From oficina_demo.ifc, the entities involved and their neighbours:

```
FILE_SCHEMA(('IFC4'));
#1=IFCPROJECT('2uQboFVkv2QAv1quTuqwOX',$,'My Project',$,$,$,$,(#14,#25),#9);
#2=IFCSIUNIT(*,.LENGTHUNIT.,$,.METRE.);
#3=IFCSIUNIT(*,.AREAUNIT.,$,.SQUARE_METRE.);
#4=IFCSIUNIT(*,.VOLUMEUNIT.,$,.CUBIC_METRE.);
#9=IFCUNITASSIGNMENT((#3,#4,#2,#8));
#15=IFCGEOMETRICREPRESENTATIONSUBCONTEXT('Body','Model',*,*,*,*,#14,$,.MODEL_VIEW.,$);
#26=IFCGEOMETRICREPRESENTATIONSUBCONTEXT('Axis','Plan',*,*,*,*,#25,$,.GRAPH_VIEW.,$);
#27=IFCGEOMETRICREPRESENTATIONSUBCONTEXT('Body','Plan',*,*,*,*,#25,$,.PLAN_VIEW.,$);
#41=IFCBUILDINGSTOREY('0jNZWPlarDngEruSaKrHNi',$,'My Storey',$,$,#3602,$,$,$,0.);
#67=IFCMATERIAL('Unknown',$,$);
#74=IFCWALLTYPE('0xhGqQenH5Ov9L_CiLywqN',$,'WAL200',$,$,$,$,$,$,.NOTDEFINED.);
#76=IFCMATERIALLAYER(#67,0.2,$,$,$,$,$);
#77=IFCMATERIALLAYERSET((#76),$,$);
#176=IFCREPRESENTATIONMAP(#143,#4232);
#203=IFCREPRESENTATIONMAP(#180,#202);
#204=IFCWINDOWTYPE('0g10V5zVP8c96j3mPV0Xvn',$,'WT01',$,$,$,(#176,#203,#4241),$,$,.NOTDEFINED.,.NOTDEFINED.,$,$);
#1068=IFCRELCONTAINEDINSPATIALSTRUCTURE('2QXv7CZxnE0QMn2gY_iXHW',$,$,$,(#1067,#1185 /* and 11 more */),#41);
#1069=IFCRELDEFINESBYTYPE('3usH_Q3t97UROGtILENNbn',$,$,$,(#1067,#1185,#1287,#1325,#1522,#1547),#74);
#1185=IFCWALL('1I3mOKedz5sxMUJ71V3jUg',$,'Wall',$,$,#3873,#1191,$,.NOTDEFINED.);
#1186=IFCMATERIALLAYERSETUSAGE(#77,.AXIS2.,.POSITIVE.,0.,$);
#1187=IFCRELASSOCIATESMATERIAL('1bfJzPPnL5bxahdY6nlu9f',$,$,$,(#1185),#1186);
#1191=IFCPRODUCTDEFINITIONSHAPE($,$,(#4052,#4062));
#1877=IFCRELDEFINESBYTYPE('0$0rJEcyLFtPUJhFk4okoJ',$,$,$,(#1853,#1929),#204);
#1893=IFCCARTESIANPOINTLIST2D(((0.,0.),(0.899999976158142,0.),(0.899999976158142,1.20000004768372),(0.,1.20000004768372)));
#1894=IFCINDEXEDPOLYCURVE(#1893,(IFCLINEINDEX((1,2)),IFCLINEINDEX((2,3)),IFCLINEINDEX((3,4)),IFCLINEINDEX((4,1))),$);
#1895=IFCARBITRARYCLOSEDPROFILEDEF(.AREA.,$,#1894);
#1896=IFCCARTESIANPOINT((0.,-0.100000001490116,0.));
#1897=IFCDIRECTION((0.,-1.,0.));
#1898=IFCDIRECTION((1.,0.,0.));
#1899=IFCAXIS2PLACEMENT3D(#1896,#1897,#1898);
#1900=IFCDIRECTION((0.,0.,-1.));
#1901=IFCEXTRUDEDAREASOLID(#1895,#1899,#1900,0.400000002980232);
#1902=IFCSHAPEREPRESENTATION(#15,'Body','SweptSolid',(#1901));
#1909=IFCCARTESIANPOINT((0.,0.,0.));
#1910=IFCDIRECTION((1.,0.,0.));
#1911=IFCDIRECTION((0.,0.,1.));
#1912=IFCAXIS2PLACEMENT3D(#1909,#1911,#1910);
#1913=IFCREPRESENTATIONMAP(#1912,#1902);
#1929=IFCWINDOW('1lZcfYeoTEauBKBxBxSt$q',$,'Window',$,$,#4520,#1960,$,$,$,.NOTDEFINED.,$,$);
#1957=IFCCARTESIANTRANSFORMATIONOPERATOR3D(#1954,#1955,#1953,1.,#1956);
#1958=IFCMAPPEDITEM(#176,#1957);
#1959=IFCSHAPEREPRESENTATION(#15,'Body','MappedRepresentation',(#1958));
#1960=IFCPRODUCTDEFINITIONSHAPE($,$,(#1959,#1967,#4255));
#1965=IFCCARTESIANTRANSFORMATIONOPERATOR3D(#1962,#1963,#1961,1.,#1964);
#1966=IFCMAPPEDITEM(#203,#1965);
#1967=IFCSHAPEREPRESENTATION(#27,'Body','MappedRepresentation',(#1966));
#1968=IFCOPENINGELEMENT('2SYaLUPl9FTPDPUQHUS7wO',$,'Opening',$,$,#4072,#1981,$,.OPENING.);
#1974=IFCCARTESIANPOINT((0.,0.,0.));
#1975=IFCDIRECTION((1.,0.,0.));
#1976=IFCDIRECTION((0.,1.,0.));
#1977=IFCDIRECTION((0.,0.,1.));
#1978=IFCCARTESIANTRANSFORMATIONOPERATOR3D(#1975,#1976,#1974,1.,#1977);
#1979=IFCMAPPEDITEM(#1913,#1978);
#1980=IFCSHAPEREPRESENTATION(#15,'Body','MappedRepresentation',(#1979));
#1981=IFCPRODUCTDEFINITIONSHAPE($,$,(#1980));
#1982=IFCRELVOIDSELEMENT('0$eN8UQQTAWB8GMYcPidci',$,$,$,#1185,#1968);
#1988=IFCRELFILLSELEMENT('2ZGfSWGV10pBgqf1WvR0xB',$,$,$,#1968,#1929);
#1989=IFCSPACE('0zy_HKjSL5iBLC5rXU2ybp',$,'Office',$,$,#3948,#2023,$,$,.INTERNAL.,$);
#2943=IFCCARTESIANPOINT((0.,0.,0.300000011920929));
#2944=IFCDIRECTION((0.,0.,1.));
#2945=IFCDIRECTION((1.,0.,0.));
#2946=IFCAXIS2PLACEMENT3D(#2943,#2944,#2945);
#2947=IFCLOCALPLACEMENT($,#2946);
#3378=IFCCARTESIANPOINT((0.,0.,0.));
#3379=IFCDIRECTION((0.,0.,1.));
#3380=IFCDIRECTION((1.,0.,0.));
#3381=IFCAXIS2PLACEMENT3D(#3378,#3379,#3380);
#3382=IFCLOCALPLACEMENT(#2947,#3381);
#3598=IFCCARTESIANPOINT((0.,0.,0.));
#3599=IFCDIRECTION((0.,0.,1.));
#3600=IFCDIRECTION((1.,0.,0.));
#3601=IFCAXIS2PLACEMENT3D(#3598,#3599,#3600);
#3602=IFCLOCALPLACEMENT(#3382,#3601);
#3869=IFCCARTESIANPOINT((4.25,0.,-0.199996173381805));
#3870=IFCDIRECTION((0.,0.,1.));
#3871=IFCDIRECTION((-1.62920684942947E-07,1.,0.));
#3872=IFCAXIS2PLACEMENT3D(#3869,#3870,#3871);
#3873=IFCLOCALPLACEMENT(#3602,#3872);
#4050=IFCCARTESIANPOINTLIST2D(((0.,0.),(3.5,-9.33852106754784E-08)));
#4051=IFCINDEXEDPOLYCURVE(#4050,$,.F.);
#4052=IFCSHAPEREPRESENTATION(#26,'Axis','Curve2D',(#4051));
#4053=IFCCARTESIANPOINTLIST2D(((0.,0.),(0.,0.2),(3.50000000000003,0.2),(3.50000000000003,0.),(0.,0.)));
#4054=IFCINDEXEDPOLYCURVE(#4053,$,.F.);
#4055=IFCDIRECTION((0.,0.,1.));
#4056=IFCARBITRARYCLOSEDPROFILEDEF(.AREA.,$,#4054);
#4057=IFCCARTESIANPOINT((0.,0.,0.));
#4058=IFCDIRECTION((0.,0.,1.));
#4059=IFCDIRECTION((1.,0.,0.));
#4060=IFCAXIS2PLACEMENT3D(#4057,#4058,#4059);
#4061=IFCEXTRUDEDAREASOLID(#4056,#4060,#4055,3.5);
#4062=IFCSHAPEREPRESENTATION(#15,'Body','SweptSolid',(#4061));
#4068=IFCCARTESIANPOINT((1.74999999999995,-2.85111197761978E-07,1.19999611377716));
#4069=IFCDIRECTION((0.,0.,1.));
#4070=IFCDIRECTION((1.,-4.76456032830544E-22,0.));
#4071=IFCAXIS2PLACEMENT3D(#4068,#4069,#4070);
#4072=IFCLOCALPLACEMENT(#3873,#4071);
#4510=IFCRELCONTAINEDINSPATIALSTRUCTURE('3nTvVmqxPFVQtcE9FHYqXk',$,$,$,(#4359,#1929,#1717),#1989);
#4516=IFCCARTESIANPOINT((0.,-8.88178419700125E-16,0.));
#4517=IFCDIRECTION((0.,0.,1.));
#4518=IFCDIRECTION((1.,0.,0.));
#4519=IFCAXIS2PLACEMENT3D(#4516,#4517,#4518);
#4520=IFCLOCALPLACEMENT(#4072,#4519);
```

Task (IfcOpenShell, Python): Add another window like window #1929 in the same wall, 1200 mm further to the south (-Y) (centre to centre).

```python
import ifcopenshell
import ifcopenshell.api.feature
import ifcopenshell.api.geometry
import ifcopenshell.api.root
import ifcopenshell.geom
import ifcopenshell.util.element
import ifcopenshell.util.placement
import ifcopenshell.util.shape

model = ifcopenshell.open("oficina_demo.ifc")
settings = ifcopenshell.geom.settings()


def volume(element):
    """Net volume in cubic metres, openings subtracted."""
    shape = ifcopenshell.geom.create_shape(settings, element)
    return ifcopenshell.util.shape.get_volume(shape.geometry)


window = model.by_guid("1lZcfYeoTEauBKBxBxSt$q")
opening = window.FillsVoids[0].RelatingOpeningElement
wall = opening.VoidsElements[0].RelatingBuildingElement
before = volume(wall)
shift = ifcopenshell.util.placement.get_local_placement(wall.ObjectPlacement)[:3, 0] * -1.2

# copy_class copies the void relationship, type, container and properties, but no geometry.
new_opening = ifcopenshell.api.root.copy_class(model, product=opening)
new_opening.Representation = ifcopenshell.util.element.copy_deep(
    model, opening.Representation, exclude=["IfcGeometricRepresentationContext", "IfcRepresentationMap"]
)
new_window = ifcopenshell.api.root.copy_class(model, product=window)
new_window.Representation = ifcopenshell.util.element.copy_deep(
    model, window.Representation, exclude=["IfcGeometricRepresentationContext", "IfcRepresentationMap"]
)
ifcopenshell.api.feature.add_filling(model, opening=new_opening, element=new_window)

for old, new in ((opening, new_opening), (window, new_window)):
    matrix = ifcopenshell.util.placement.get_local_placement(old.ObjectPlacement)
    matrix[:3, 3] += shift
    ifcopenshell.api.geometry.edit_object_placement(model, product=new, matrix=matrix, is_si=False)

after = volume(wall)

print(f"wall volume {before:.3f} -> {after:.3f} m3")

model.write("oficina_demo_rev.ifc")
```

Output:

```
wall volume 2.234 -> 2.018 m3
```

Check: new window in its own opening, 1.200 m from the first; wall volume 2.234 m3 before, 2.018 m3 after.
